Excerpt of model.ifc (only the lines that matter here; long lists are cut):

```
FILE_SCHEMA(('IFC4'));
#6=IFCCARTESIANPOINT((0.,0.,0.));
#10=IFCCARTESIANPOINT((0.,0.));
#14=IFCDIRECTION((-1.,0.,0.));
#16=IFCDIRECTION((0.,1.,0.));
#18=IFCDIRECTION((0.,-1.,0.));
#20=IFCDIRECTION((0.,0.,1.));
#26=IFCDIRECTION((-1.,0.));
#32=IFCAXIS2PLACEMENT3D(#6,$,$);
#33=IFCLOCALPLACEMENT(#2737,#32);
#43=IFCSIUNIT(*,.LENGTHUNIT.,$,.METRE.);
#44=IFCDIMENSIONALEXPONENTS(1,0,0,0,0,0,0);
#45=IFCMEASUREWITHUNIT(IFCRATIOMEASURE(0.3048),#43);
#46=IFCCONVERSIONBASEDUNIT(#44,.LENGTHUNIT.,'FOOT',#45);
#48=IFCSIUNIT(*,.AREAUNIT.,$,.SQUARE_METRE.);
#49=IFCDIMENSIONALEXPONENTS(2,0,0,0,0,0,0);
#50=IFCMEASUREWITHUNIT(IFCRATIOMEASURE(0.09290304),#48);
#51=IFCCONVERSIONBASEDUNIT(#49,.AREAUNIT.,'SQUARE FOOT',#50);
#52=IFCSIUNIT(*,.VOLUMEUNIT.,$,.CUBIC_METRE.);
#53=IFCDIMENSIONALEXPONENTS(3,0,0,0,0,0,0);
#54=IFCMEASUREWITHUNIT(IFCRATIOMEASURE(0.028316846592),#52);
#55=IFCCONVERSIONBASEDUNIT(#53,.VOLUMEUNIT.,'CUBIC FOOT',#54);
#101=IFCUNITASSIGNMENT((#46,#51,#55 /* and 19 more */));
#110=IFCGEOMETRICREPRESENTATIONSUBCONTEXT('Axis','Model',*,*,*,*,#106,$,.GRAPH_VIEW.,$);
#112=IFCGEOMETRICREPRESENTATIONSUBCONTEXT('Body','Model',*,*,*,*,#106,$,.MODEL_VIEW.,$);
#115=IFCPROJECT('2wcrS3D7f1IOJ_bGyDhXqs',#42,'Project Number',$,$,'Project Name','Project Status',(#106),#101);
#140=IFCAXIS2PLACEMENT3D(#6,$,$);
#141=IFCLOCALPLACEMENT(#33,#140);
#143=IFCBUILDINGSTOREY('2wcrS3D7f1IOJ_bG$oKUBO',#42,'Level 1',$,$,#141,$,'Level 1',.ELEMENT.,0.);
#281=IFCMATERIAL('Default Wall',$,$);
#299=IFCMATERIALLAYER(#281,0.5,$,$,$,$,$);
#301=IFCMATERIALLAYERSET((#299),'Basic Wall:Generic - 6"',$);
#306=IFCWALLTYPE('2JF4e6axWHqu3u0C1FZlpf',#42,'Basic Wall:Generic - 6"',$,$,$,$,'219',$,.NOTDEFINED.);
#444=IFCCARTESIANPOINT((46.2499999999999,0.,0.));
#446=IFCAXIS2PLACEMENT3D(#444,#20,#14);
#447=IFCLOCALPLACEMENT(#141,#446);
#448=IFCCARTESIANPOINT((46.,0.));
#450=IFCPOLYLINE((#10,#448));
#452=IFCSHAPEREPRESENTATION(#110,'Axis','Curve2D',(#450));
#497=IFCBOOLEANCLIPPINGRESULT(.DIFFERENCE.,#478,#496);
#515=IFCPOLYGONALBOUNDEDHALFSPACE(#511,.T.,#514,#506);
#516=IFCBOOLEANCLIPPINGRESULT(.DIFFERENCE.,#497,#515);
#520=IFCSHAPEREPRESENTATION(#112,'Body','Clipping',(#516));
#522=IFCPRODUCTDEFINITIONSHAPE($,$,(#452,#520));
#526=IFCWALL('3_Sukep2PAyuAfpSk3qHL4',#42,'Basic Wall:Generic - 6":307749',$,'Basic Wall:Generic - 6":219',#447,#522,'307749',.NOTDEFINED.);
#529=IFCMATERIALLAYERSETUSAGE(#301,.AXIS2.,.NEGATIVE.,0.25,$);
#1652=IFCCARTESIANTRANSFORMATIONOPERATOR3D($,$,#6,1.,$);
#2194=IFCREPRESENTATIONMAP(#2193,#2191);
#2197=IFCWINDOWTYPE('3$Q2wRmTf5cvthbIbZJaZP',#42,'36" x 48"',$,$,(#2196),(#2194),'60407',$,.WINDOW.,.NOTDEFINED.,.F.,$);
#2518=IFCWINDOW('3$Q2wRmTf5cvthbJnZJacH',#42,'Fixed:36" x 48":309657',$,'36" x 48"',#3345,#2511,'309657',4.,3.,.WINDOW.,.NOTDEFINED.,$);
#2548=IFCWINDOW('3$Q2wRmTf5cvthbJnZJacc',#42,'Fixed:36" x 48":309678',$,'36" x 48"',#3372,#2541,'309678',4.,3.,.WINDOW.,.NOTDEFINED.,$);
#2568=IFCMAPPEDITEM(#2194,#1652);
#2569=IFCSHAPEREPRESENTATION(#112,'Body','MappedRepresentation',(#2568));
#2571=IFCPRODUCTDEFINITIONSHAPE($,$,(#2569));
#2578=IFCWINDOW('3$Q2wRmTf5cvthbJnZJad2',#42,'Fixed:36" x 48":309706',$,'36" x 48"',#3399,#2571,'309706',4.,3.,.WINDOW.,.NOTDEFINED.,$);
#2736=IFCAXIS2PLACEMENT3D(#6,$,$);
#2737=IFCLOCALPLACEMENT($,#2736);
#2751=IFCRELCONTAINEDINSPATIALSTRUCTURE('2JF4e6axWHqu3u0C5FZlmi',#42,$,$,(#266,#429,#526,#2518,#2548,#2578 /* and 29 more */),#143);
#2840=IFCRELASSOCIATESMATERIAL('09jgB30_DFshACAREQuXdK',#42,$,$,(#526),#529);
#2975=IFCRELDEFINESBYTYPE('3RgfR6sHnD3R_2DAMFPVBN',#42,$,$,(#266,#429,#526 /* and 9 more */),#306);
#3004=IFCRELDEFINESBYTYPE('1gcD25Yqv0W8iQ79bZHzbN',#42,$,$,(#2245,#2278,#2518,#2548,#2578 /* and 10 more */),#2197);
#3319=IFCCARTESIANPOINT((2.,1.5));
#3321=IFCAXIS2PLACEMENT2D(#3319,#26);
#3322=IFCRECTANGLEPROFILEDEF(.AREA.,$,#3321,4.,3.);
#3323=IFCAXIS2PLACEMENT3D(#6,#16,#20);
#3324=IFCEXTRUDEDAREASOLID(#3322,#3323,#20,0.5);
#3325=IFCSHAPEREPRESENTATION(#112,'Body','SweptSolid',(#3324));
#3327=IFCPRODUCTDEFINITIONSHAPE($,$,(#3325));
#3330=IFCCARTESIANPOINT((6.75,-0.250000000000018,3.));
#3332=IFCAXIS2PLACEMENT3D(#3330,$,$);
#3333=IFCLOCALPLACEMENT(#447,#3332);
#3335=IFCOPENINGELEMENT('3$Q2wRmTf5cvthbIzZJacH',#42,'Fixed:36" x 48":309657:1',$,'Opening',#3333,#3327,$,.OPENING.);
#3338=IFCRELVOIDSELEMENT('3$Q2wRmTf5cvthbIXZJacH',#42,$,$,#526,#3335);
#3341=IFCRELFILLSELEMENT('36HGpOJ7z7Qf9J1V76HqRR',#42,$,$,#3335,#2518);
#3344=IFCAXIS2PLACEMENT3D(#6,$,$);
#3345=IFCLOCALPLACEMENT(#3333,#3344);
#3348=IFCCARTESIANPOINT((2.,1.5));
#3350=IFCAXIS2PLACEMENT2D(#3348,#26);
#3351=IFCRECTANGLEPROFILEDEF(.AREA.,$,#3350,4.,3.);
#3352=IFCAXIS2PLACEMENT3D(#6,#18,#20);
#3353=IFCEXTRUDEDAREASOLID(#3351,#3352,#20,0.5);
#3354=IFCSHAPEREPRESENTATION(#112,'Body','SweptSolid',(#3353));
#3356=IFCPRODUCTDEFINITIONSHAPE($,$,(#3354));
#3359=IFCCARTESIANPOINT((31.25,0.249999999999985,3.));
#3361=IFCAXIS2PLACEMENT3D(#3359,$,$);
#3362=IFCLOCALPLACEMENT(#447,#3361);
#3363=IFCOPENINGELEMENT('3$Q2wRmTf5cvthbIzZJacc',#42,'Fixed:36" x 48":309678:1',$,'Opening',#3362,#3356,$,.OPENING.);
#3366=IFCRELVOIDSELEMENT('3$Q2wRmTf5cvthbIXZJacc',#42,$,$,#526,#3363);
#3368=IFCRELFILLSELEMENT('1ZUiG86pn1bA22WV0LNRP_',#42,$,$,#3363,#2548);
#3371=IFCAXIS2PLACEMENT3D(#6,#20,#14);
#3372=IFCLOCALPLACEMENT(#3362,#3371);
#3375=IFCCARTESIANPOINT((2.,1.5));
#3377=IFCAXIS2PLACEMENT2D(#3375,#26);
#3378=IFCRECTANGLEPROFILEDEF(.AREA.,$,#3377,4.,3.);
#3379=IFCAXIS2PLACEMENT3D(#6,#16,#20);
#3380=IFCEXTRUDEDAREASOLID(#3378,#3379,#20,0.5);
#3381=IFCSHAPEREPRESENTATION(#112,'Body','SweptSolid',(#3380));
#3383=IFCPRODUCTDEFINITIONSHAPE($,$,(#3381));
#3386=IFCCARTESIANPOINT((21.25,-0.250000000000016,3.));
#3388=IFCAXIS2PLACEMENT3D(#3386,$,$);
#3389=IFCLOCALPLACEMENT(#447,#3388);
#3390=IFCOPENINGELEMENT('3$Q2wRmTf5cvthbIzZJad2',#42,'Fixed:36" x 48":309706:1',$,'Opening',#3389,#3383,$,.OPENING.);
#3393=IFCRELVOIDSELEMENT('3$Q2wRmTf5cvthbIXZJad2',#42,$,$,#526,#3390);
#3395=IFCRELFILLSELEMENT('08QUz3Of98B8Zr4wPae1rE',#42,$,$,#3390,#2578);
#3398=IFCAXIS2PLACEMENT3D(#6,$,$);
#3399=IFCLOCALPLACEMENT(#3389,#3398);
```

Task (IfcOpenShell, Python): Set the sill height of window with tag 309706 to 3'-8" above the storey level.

```python
import numpy as np
import ifcopenshell
import ifcopenshell.api.geometry
import ifcopenshell.geom
import ifcopenshell.util.element
import ifcopenshell.util.placement
import ifcopenshell.util.shape
import ifcopenshell.util.unit

model = ifcopenshell.open("model.ifc")
unit_scale = ifcopenshell.util.unit.calculate_unit_scale(model)

window = model.by_guid("3$Q2wRmTf5cvthbJnZJad2")
opening = window.FillsVoids[0].RelatingOpeningElement
storey = ifcopenshell.util.element.get_container(window, ifc_class="IfcBuildingStorey")
level = ifcopenshell.util.placement.get_local_placement(storey.ObjectPlacement)[2, 3]

# The opening's origin need not be at the sill, so measure its lowest point.
shape = ifcopenshell.geom.create_shape(ifcopenshell.geom.settings(), opening)
bottom = ifcopenshell.util.shape.get_shape_bottom_elevation(shape, shape.geometry) / unit_scale
dz = level + 44 * 0.0254 / unit_scale - bottom

shift = np.array([0.0, 0.0, dz])
# The window is placed relative to its opening, so it follows when the opening moves.
matrix = ifcopenshell.util.placement.get_local_placement(opening.ObjectPlacement)
matrix[:3, 3] += shift
ifcopenshell.api.geometry.edit_object_placement(
    model, product=opening, matrix=matrix, is_si=False, should_transform_children=True
)

print(f"moved by {dz * unit_scale:+.3f} m")

model.write("model_rev.ifc")
```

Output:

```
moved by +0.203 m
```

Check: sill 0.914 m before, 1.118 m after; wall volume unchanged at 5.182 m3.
